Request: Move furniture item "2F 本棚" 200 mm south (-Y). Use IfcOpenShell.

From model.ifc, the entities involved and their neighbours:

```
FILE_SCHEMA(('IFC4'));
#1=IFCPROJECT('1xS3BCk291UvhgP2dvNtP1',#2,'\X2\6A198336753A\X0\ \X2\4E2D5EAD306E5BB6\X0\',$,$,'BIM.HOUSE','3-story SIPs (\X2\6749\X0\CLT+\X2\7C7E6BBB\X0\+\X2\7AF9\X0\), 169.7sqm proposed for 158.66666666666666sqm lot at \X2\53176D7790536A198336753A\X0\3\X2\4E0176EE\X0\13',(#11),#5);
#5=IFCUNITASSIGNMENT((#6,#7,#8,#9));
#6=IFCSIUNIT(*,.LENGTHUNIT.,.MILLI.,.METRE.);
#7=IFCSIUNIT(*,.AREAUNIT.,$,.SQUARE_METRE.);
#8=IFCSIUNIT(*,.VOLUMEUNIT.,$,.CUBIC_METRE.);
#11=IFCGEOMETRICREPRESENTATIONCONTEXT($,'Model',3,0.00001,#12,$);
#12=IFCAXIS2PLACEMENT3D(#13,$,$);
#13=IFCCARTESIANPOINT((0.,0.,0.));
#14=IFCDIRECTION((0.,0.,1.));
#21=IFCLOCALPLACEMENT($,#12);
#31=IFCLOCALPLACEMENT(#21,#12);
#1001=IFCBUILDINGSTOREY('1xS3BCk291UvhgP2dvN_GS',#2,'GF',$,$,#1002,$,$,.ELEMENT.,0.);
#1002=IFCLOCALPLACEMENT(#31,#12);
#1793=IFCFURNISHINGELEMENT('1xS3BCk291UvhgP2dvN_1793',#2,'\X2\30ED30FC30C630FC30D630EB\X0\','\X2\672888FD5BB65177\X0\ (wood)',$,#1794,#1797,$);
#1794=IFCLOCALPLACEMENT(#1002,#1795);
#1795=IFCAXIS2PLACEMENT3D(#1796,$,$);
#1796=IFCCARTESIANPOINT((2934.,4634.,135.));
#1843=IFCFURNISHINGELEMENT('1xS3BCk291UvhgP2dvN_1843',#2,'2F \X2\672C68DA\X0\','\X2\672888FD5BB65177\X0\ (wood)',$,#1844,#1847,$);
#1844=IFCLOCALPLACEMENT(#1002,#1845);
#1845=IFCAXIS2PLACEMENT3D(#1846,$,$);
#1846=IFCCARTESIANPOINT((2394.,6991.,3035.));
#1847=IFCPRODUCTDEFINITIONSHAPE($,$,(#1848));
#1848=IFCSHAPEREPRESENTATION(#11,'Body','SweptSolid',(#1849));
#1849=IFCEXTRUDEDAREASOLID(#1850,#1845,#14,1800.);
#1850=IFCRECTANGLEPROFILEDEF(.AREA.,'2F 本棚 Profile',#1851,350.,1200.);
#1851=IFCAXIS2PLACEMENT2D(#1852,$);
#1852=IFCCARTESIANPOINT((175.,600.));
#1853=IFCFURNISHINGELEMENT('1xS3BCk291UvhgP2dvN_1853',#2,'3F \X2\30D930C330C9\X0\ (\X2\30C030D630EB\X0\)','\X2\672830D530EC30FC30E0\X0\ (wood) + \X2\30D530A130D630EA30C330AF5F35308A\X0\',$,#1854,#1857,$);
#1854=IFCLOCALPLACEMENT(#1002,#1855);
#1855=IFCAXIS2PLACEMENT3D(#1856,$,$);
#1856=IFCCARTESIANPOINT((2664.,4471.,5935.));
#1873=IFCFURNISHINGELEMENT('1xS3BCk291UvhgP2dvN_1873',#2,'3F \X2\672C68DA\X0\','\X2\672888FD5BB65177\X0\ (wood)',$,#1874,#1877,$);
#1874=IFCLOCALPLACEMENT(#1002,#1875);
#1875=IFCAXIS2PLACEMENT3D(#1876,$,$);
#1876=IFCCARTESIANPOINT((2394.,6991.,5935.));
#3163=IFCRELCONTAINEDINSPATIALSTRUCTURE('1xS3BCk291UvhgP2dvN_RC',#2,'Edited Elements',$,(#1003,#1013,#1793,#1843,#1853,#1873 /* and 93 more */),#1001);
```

```python
import ifcopenshell
import ifcopenshell.api.geometry
import ifcopenshell.util.placement

model = ifcopenshell.open("model.ifc")

item = model.by_id(1843)
matrix = ifcopenshell.util.placement.get_local_placement(item.ObjectPlacement)
matrix[1, 3] -= 200.0
ifcopenshell.api.geometry.edit_object_placement(model, product=item, matrix=matrix, is_si=False)

print(ifcopenshell.util.placement.get_local_placement(item.ObjectPlacement).round(3) + 0.0)

model.write("model_updated.ifc")
```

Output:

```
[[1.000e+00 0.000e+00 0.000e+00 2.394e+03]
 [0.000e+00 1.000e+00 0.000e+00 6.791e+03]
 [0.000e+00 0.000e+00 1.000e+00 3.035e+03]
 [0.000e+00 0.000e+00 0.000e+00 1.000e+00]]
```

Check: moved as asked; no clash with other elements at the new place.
